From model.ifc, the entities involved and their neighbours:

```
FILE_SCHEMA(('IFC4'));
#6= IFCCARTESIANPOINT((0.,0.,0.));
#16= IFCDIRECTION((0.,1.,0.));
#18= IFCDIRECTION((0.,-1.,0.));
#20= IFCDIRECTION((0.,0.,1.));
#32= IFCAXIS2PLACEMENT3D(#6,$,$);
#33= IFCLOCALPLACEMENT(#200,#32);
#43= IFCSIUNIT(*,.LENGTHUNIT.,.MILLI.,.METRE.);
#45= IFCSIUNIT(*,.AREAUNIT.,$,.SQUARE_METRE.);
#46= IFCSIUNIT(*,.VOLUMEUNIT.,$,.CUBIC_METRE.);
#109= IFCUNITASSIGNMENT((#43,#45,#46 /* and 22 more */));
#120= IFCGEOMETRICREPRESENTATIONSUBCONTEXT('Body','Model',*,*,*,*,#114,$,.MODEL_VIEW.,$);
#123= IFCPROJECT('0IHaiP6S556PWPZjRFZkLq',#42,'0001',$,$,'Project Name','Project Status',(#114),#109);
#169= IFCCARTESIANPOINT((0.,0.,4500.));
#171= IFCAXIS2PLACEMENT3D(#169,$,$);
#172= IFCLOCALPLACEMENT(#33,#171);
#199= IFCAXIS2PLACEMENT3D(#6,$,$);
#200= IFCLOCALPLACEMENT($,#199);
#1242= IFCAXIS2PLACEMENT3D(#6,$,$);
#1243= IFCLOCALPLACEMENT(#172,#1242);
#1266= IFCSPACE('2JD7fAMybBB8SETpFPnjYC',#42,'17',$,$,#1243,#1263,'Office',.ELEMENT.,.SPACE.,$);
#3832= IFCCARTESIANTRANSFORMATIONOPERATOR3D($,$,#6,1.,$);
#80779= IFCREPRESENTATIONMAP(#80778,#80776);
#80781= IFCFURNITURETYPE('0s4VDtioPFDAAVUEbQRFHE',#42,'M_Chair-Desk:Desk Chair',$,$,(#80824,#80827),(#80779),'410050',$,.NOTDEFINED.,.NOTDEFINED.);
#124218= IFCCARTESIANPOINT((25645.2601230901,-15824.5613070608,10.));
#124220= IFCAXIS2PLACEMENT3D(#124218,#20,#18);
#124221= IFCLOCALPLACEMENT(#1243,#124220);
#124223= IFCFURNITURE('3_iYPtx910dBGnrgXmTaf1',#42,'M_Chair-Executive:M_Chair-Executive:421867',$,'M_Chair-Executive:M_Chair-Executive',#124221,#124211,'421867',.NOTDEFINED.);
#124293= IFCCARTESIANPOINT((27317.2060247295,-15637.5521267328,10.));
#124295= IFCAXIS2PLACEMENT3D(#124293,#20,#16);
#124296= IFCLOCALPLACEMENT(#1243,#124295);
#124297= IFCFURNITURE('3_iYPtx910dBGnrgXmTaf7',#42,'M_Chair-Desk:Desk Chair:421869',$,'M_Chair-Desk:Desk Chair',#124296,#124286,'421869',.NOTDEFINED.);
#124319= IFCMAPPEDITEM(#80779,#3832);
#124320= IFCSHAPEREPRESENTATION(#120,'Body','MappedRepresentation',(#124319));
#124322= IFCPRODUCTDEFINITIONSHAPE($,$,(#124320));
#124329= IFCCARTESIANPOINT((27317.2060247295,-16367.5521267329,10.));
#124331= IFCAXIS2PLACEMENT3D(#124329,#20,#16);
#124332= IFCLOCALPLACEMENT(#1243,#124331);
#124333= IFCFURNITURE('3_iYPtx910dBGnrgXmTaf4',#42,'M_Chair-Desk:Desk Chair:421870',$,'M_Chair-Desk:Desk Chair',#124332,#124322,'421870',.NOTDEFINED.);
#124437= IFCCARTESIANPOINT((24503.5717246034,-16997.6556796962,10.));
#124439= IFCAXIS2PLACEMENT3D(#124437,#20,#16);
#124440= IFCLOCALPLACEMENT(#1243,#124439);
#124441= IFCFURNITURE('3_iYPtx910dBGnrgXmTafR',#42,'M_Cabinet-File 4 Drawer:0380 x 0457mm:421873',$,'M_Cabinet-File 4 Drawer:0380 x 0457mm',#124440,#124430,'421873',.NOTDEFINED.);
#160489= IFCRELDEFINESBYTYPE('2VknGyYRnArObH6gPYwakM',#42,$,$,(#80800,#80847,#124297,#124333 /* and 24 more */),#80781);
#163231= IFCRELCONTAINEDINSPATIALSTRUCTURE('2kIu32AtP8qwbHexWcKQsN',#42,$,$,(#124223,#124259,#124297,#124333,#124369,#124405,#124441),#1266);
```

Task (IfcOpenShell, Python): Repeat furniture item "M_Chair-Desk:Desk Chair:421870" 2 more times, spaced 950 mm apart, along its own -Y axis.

```python
import ifcopenshell
import ifcopenshell.api.geometry
import ifcopenshell.api.root
import ifcopenshell.util.element
import ifcopenshell.util.placement
import ifcopenshell.util.unit

model = ifcopenshell.open("model.ifc")
unit_scale = ifcopenshell.util.unit.calculate_unit_scale(model)


def reuse_history(source, copy):
    """copy_class also copies each property set's owner history, people and application; keep the originals."""
    for rel in copy.IsDefinedBy:
        if rel.is_a("IfcRelDefinesByProperties") and (history := rel.RelatingPropertyDefinition.OwnerHistory):
            rel.RelatingPropertyDefinition.OwnerHistory = source.OwnerHistory
            ifcopenshell.util.element.remove_deep2(model, history)


source = model.by_guid("3_iYPtx910dBGnrgXmTaf4")
base = ifcopenshell.util.placement.get_local_placement(source.ObjectPlacement)
step = -base[:3, 1] * 0.95 / unit_scale

for i in range(1, 3):
    copy = ifcopenshell.api.root.copy_class(model, product=source)
    copy.Representation = ifcopenshell.util.element.copy_deep(
        model, source.Representation, exclude=["IfcGeometricRepresentationContext", "IfcRepresentationMap"]
    )
    copy.Name = "M_Chair-Desk:Desk Chair"
    copy.Tag = None
    reuse_history(source, copy)
    matrix = base.copy()
    matrix[:3, 3] += i * step
    print("added at", matrix[:3, 3].round(3) + 0.0)
    ifcopenshell.api.geometry.edit_object_placement(model, product=copy, matrix=matrix, is_si=False)

model.write("model-out.ifc")
```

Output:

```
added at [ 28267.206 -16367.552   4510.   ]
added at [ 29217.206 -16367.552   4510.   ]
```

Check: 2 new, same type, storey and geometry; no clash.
